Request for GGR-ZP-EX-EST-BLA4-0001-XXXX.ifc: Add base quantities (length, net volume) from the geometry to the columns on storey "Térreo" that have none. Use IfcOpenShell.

First a look at what the model holds.

```python
import ifcopenshell
import ifcopenshell.util.element
import ifcopenshell.util.unit

model = ifcopenshell.open("GGR-ZP-EX-EST-BLA4-0001-XXXX.ifc")
print(model.schema)
for unit_type in ("LENGTHUNIT", "AREAUNIT", "VOLUMEUNIT"):
    print(unit_type, ifcopenshell.util.unit.calculate_unit_scale(model, unit_type))
storey = next(s for s in model.by_type("IfcBuildingStorey") if s.Name == "Térreo")
columns = [e for e in ifcopenshell.util.element.get_decomposition(storey) if e.is_a("IfcColumn")]
for e in sorted(columns, key=lambda e: e.id()):
    print(e.id(), e.is_a(), e.Name, list(ifcopenshell.util.element.get_psets(e, qtos_only=True)), sep=" | ")
```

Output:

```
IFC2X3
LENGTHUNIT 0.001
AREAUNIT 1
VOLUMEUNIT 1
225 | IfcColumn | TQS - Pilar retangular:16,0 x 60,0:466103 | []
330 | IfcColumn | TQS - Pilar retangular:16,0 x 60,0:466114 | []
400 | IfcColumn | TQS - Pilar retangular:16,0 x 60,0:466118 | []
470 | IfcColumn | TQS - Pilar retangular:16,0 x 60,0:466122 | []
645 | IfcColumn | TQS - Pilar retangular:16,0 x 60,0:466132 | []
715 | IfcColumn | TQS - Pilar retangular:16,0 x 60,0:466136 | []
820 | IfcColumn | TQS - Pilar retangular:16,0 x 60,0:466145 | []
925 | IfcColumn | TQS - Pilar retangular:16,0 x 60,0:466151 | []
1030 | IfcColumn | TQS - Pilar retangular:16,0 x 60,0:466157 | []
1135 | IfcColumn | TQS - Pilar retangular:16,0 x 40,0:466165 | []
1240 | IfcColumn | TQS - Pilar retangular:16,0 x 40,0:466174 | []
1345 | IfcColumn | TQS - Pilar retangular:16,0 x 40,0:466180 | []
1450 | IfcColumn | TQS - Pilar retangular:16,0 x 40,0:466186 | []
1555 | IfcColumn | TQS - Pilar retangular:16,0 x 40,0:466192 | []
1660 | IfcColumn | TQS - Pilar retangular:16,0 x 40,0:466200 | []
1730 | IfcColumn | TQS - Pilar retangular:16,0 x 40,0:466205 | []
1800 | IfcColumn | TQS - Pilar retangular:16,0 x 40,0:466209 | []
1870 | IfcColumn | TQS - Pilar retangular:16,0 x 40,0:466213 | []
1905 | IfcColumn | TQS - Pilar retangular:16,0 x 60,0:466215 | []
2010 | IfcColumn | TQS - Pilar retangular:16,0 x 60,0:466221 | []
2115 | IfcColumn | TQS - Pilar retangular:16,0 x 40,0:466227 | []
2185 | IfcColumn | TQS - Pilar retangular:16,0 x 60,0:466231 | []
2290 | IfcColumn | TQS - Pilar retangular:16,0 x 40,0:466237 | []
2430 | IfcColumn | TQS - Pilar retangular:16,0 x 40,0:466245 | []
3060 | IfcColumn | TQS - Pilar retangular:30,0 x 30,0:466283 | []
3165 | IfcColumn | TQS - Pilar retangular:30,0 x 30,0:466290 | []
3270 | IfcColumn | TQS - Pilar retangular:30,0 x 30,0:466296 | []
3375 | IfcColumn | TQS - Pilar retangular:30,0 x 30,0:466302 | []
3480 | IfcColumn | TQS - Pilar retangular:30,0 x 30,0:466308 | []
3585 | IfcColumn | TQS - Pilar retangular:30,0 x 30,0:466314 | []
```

```python
import ifcopenshell
import ifcopenshell.api.pset
import ifcopenshell.geom
import ifcopenshell.util.element
import ifcopenshell.util.shape
import ifcopenshell.util.unit

model = ifcopenshell.open("GGR-ZP-EX-EST-BLA4-0001-XXXX.ifc")
unit_scale = ifcopenshell.util.unit.calculate_unit_scale(model)
volume_scale = ifcopenshell.util.unit.calculate_unit_scale(model, "VOLUMEUNIT")
settings = ifcopenshell.geom.settings()

storey = next(s for s in model.by_type("IfcBuildingStorey") if s.Name == "Térreo")
columns = [e for e in ifcopenshell.util.element.get_decomposition(storey) if e.is_a("IfcColumn")]

for e in sorted(columns, key=lambda e: e.id()):
    if ifcopenshell.util.element.get_psets(e, qtos_only=True, should_inherit=False):
        continue
    # Geometry comes back in metres, in the element's own axes.
    shape = ifcopenshell.geom.create_shape(settings, e)
    values = {
        "Length": ifcopenshell.util.shape.get_z(shape.geometry) / unit_scale,
        "NetVolume": ifcopenshell.util.shape.get_volume(shape.geometry) / volume_scale,
    }
    qto = ifcopenshell.api.pset.add_qto(model, product=e, name="BaseQuantities")
    ifcopenshell.api.pset.edit_qto(model, qto=qto, properties=values)
    print(e.id(), {k: round(v, 3) for k, v in values.items()})

model.write("GGR-ZP-EX-EST-BLA4-0001-XXXX_edited.ifc")
```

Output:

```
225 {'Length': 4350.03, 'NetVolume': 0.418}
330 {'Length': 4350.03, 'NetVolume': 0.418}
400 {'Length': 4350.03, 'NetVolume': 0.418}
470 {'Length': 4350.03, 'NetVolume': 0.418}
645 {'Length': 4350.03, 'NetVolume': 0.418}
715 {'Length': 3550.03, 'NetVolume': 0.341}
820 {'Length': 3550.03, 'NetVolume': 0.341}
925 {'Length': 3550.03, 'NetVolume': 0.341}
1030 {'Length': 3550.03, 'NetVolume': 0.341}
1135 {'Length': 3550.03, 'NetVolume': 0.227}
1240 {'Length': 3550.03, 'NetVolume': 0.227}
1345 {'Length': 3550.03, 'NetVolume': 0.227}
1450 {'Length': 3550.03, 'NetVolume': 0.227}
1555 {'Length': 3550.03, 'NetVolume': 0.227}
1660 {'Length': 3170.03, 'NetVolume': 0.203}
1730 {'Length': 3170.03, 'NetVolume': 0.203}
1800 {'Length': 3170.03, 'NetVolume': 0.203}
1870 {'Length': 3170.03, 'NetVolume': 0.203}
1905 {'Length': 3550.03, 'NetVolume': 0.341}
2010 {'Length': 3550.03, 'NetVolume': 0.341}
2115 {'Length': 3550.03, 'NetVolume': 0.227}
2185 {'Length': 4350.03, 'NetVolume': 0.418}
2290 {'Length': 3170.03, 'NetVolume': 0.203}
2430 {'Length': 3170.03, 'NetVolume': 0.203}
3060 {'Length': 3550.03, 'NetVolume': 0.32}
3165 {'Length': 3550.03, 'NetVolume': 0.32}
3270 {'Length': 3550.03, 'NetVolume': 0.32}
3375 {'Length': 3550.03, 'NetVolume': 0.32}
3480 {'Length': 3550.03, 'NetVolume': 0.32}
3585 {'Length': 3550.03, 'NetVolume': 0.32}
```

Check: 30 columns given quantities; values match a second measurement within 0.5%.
